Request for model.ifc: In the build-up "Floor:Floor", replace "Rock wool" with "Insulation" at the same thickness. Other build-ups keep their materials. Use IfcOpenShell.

First a look at what the model holds.

```python
import ifcopenshell
import ifcopenshell.util.element

model = ifcopenshell.open("model.ifc")
print(model.schema)
for layer_set in model.by_type("IfcMaterialLayerSet"):
    if layer_set.LayerSetName == "Floor:Floor":
        for layer in layer_set.MaterialLayers:
            print(layer.id(), layer.Material and layer.Material.Name, layer.LayerThickness, sep=" | ")
        print(len(ifcopenshell.util.element.get_elements_by_material(model, layer_set)), "elements and types use it")
print(sorted(m.Name for m in model.by_type("IfcMaterial") if m.Name)[:60])
```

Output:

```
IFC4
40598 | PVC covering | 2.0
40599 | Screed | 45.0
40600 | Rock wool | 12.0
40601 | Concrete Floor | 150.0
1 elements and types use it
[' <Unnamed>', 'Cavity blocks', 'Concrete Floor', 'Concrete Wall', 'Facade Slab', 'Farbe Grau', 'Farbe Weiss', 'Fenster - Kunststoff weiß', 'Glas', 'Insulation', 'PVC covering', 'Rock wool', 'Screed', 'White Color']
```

```python
import ifcopenshell
import ifcopenshell.api.material

model = ifcopenshell.open("model.ifc")

layer_set = next(s for s in model.by_type("IfcMaterialLayerSet") if s.LayerSetName == "Floor:Floor")
layer = next(l for l in layer_set.MaterialLayers if l.Material and l.Material.Name == "Rock wool")
material = next(m for m in model.by_type("IfcMaterial") if m.Name == "Insulation")

# Point this one layer at the other material; renaming the old one would change it everywhere.
ifcopenshell.api.material.edit_layer(model, layer=layer, attributes={}, material=material)

print([l.Material.Name if l.Material else None for l in layer_set.MaterialLayers])

model.write("model_edited.ifc")
```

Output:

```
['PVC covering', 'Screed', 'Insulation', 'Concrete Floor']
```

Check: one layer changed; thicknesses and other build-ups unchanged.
